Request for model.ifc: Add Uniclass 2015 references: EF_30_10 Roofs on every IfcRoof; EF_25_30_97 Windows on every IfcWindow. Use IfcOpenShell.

First a look at what the model holds.

```python
import ifcopenshell

model = ifcopenshell.open("model.ifc")
print(model.schema)
print("classifications:", [c.Name for c in model.by_type("IfcClassification")])
for ifc_class in ("IfcDoor", "IfcRoof", "IfcStair", "IfcWall", "IfcWindow"):
    print(ifc_class, len(model.by_type(ifc_class)))
```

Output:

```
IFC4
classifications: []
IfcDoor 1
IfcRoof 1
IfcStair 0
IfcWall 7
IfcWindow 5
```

```python
import ifcopenshell
import ifcopenshell.api.classification

model = ifcopenshell.open("model.ifc")

system = ifcopenshell.api.classification.add_classification(model, classification="Uniclass 2015")

codes = {
    "IfcRoof": ("EF_30_10", "Roofs"),
    "IfcWindow": ("EF_25_30_97", "Windows"),
}
for ifc_class, (code, name) in codes.items():
    products = model.by_type(ifc_class)
    ifcopenshell.api.classification.add_reference(
        model, products=products, classification=system, identification=code, name=name
    )
    print(code, len(products))

model.write("model-out.ifc")
```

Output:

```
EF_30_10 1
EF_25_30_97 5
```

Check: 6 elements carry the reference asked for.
